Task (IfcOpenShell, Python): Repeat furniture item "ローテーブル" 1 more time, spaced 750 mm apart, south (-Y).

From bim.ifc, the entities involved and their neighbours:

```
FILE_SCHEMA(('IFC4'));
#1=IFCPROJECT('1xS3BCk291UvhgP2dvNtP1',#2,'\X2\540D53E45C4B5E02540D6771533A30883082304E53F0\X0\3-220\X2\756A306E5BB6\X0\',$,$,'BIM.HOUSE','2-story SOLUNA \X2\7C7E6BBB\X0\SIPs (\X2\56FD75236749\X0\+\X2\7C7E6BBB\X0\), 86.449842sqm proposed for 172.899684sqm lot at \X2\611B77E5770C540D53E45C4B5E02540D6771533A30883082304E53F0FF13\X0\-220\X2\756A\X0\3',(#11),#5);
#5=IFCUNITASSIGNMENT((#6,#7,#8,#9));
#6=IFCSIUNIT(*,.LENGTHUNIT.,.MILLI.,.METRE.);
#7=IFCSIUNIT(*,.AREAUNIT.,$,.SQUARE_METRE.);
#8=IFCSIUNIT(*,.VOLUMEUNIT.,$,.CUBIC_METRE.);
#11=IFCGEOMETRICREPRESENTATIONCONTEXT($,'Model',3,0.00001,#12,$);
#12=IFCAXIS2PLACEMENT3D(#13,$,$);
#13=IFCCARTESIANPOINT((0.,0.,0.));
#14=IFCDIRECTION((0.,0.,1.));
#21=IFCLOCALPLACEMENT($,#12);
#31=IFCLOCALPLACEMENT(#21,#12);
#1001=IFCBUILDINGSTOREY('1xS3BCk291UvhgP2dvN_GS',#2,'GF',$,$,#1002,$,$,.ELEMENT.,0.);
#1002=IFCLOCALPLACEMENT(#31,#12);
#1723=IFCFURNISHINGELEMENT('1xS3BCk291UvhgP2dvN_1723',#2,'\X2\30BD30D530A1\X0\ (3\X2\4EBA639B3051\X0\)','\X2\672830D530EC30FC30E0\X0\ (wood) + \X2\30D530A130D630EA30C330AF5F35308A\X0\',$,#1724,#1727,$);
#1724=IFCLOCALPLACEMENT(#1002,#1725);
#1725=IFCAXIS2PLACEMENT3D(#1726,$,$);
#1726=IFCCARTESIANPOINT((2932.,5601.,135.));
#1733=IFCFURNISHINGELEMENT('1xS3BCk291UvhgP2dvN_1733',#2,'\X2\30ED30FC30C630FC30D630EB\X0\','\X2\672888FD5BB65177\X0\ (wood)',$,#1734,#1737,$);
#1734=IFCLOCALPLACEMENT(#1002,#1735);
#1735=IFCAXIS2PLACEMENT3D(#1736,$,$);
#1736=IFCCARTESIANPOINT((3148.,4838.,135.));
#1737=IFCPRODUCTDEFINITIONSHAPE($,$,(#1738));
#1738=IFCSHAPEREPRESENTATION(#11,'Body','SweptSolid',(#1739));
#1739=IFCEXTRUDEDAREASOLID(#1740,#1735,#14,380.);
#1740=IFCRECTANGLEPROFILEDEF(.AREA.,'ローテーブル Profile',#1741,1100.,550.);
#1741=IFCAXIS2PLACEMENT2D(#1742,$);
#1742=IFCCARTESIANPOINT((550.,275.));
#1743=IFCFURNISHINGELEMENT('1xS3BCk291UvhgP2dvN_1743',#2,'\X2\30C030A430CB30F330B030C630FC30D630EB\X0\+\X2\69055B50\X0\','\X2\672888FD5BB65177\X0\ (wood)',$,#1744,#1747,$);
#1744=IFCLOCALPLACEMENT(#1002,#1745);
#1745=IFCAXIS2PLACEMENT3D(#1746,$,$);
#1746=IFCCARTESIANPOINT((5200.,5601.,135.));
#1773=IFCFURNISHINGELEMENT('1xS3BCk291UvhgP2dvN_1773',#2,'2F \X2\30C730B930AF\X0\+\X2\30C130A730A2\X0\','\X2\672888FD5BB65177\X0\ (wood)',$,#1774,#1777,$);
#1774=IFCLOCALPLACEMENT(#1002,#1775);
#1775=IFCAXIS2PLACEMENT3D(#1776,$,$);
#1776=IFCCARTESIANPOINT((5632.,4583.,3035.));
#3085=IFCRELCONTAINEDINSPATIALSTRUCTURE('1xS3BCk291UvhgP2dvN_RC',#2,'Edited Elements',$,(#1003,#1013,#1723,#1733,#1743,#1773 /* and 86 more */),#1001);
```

```python
import numpy as np
import ifcopenshell
import ifcopenshell.api.geometry
import ifcopenshell.api.root
import ifcopenshell.util.element
import ifcopenshell.util.placement

model = ifcopenshell.open("bim.ifc")


def reuse_history(source, copy):
    """copy_class also copies each property set's owner history, people and application; keep the originals."""
    for rel in copy.IsDefinedBy:
        if rel.is_a("IfcRelDefinesByProperties") and (history := rel.RelatingPropertyDefinition.OwnerHistory):
            rel.RelatingPropertyDefinition.OwnerHistory = source.OwnerHistory
            ifcopenshell.util.element.remove_deep2(model, history)


source = model.by_guid("1xS3BCk291UvhgP2dvN_1733")
base = ifcopenshell.util.placement.get_local_placement(source.ObjectPlacement)
step = np.array([0.0, -1.0, 0.0]) * 750.0

for i in range(1, 2):
    copy = ifcopenshell.api.root.copy_class(model, product=source)
    copy.Representation = ifcopenshell.util.element.copy_deep(
        model, source.Representation, exclude=["IfcGeometricRepresentationContext", "IfcRepresentationMap"]
    )
    reuse_history(source, copy)
    matrix = base.copy()
    matrix[:3, 3] += i * step
    print("added at", matrix[:3, 3].round(3) + 0.0)
    ifcopenshell.api.geometry.edit_object_placement(model, product=copy, matrix=matrix, is_si=False)

model.write("bim_v2.ifc")
```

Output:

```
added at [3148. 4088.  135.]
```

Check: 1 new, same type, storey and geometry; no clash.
